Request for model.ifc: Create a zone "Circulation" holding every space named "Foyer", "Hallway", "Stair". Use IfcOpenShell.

First a look at what the model holds.

```python
import ifcopenshell

model = ifcopenshell.open("model.ifc")
print(model.schema)
seen = {}
for space in model.by_type("IfcSpace"):
    seen[space.LongName] = seen.get(space.LongName, 0) + 1
for name, count in sorted(seen.items(), key=str):
    print(count, "x", name)
print("zones:", [z.Name for z in model.by_type("IfcZone")][:20])
```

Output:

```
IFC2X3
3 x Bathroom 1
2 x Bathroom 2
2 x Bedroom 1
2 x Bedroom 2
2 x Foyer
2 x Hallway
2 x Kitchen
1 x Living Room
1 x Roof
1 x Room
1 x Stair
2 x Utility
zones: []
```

```python
import ifcopenshell
import ifcopenshell.api.group
import ifcopenshell.api.root

model = ifcopenshell.open("model.ifc")

names = {"Foyer", "Hallway", "Stair"}
spaces = [s for s in model.by_type("IfcSpace") if s.LongName in names]

zone = ifcopenshell.api.root.create_entity(model, ifc_class="IfcZone", name="Circulation")
ifcopenshell.api.group.assign_group(model, products=spaces, group=zone)
print(len(spaces), "spaces in", zone.Name)

model.write("model_updated.ifc")
```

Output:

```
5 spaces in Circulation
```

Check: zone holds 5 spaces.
